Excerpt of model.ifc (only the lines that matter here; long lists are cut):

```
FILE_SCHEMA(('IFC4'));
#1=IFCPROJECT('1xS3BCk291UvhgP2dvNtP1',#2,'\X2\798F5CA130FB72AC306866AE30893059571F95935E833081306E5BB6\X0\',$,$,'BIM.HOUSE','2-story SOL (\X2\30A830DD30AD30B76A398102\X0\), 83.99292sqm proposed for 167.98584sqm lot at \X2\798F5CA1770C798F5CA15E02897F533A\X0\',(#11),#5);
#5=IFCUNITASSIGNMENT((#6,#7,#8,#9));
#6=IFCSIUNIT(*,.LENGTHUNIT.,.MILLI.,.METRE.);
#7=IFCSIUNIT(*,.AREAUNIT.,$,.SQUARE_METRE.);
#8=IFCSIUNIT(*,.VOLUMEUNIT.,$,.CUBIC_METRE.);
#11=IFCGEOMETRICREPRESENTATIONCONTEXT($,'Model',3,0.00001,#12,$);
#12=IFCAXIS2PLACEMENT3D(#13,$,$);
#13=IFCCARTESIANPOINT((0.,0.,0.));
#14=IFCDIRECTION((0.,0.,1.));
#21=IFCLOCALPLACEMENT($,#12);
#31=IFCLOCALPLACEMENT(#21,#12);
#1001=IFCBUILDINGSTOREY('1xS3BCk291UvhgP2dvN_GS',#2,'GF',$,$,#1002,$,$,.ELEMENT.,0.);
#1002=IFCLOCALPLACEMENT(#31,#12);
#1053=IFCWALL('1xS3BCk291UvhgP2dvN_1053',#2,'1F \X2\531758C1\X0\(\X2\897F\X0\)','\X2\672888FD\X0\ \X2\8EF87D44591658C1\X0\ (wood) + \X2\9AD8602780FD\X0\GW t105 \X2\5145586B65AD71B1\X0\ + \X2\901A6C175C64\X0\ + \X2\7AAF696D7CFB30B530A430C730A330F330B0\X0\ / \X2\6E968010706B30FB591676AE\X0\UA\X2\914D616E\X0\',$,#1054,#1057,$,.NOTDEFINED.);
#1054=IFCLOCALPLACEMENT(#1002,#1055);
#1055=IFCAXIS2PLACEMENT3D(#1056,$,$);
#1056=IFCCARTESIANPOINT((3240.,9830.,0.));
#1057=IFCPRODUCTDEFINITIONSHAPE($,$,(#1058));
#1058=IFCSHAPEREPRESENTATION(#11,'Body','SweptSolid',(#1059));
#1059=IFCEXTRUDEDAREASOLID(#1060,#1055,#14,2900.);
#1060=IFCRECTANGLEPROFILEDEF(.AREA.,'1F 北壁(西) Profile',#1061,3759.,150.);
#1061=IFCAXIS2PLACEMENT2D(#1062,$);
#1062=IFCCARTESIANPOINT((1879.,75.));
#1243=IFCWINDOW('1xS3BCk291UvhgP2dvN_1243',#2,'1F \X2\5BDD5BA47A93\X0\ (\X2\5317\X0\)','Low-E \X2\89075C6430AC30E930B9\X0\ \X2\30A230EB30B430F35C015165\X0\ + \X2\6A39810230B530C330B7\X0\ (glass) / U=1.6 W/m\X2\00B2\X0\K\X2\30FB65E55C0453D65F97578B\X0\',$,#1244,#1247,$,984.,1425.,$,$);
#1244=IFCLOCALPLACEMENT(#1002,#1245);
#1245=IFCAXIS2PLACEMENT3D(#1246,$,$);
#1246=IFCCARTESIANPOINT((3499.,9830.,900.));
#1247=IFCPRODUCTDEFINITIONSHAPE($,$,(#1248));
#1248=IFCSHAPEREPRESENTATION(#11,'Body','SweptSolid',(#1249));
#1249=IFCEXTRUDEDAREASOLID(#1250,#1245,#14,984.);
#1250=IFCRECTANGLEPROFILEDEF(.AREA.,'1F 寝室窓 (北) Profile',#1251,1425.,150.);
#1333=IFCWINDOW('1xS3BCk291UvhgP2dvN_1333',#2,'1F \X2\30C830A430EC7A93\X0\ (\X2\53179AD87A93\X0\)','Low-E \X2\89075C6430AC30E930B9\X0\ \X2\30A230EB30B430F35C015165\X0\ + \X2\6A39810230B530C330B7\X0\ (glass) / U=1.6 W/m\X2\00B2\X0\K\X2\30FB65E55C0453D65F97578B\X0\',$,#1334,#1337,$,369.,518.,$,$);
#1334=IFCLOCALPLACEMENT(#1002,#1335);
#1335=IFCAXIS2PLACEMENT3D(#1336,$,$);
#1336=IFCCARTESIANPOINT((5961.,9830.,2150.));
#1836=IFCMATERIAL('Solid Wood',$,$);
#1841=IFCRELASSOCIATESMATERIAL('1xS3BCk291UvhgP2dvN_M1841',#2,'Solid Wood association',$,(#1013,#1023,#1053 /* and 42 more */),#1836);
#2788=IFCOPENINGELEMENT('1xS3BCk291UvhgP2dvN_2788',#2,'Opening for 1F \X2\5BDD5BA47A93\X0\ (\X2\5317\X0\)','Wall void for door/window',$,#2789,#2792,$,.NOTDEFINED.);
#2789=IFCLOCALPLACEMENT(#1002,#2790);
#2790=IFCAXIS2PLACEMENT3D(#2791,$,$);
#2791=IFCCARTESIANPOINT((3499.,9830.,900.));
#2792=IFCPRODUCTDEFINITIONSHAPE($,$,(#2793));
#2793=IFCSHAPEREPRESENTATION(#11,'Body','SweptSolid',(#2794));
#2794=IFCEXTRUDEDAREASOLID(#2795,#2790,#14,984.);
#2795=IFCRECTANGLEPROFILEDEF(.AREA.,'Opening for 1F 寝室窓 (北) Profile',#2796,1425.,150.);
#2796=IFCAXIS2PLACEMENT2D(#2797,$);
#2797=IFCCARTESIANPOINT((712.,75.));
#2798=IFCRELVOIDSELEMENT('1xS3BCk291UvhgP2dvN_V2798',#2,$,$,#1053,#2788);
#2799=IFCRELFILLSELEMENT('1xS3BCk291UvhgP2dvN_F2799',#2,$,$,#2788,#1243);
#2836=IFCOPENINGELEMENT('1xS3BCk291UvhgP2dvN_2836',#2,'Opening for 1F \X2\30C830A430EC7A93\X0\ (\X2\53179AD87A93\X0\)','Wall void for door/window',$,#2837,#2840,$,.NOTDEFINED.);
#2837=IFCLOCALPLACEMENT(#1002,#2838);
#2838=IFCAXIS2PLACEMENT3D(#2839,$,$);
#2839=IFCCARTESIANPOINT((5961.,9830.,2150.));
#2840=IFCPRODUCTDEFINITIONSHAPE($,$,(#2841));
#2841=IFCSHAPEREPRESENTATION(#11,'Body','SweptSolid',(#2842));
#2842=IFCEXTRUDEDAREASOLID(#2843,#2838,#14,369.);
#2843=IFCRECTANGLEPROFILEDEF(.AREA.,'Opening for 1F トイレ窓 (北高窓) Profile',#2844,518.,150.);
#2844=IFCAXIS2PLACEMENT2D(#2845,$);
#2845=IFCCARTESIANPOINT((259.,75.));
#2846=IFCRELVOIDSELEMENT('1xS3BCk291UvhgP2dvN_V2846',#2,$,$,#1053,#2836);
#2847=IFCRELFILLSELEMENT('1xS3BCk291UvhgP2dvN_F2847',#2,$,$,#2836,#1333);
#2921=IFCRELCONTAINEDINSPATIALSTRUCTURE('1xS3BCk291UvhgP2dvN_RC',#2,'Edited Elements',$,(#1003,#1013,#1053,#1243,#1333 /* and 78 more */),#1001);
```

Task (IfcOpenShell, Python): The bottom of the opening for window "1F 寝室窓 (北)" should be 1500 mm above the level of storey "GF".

```python
import numpy as np
import ifcopenshell
import ifcopenshell.api.geometry
import ifcopenshell.geom
import ifcopenshell.util.element
import ifcopenshell.util.placement
import ifcopenshell.util.shape
import ifcopenshell.util.unit

model = ifcopenshell.open("model.ifc")
unit_scale = ifcopenshell.util.unit.calculate_unit_scale(model)

window = model.by_guid("1xS3BCk291UvhgP2dvN_1243")
opening = window.FillsVoids[0].RelatingOpeningElement
storey = ifcopenshell.util.element.get_container(window, ifc_class="IfcBuildingStorey")
level = ifcopenshell.util.placement.get_local_placement(storey.ObjectPlacement)[2, 3]

# The opening's origin need not be at the sill, so measure its lowest point.
shape = ifcopenshell.geom.create_shape(ifcopenshell.geom.settings(), opening)
bottom = ifcopenshell.util.shape.get_shape_bottom_elevation(shape, shape.geometry) / unit_scale
dz = level + 1.5 / unit_scale - bottom

shift = np.array([0.0, 0.0, dz])
# The window is not placed relative to its opening, so move both.
for product in (opening, window):
    matrix = ifcopenshell.util.placement.get_local_placement(product.ObjectPlacement)
    matrix[:3, 3] += shift
    ifcopenshell.api.geometry.edit_object_placement(model, product=product, matrix=matrix, is_si=False)

print(f"moved by {dz * unit_scale:+.3f} m")

model.write("model_v2.ifc")
```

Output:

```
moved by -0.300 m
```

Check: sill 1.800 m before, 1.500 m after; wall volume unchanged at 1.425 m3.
